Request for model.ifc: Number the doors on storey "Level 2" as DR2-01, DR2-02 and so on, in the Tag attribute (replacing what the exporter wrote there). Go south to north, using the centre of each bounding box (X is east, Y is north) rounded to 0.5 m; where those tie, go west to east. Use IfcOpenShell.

First a look at what the model holds.

```python
import ifcopenshell
import ifcopenshell.util.element
import ifcopenshell.util.placement

model = ifcopenshell.open("model.ifc")
print(model.schema)
storey = next(s for s in model.by_type("IfcBuildingStorey") if s.Name == "Level 2")
doors = [e for e in ifcopenshell.util.element.get_decomposition(storey) if e.is_a("IfcDoor")]
for e in sorted(doors, key=lambda e: e.id()):
    origin = ifcopenshell.util.placement.get_local_placement(e.ObjectPlacement)[:3, 3]
    print(e.id(), e.Tag, e.Name, origin.round(2) + 0.0, sep=" | ")
```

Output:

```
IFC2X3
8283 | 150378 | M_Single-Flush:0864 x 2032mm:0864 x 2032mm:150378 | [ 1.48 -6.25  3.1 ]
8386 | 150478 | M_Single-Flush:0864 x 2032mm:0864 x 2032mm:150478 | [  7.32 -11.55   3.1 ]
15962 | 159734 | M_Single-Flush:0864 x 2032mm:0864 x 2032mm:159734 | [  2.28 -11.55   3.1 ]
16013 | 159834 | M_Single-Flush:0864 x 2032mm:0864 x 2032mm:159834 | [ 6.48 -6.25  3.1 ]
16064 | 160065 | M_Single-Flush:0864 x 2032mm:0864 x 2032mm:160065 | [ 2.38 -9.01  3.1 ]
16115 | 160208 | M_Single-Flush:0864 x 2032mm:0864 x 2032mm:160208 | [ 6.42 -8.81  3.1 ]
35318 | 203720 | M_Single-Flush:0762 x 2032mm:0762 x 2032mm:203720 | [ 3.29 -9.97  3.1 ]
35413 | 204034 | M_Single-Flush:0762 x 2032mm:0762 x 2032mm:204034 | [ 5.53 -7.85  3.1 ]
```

```python
import ifcopenshell
import ifcopenshell.geom
import ifcopenshell.util.element
import ifcopenshell.util.shape

model = ifcopenshell.open("model.ifc")
settings = ifcopenshell.geom.settings()
settings.set("use-world-coords", True)


def centre(element):
    shape = ifcopenshell.geom.create_shape(settings, element)
    return ifcopenshell.util.shape.get_bbox_centroid(shape.geometry)


storey = next(s for s in model.by_type("IfcBuildingStorey") if s.Name == "Level 2")
doors = [e for e in ifcopenshell.util.element.get_decomposition(storey) if e.is_a("IfcDoor")]

# Insertion points can sit at a corner or the storey origin, so sort by the geometry (in metres).
centres = {e: centre(e) for e in doors}
doors.sort(key=lambda e: (round(centres[e][1] / 0.5), centres[e][0]))

for i, e in enumerate(doors, start=1):
    number = f"DR2-{i:02d}"
    e.Tag = number
    print(e.id(), number)

model.write("model_v2.ifc")
```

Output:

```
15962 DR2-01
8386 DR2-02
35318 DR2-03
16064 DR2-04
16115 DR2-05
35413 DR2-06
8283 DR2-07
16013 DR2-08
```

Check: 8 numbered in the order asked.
